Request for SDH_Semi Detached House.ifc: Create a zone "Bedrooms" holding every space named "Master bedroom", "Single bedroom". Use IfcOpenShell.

First a look at what the model holds.

```python
import ifcopenshell

model = ifcopenshell.open("SDH_Semi Detached House.ifc")
print(model.schema)
seen = {}
for space in model.by_type("IfcSpace"):
    seen[space.LongName] = seen.get(space.LongName, 0) + 1
for name, count in sorted(seen.items(), key=str):
    print(count, "x", name)
print("zones:", [z.Name for z in model.by_type("IfcZone")][:20])
```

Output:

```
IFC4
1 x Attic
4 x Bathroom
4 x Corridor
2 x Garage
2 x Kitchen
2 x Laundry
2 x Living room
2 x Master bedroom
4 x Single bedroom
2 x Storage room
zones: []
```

```python
import ifcopenshell
import ifcopenshell.api.group
import ifcopenshell.api.root

model = ifcopenshell.open("SDH_Semi Detached House.ifc")

names = {"Master bedroom", "Single bedroom"}
spaces = [s for s in model.by_type("IfcSpace") if s.LongName in names]

zone = ifcopenshell.api.root.create_entity(model, ifc_class="IfcZone", name="Bedrooms")
ifcopenshell.api.group.assign_group(model, products=spaces, group=zone)
print(len(spaces), "spaces in", zone.Name)

model.write("SDH_Semi Detached House_v2.ifc")
```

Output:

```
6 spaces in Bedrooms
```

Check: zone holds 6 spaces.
